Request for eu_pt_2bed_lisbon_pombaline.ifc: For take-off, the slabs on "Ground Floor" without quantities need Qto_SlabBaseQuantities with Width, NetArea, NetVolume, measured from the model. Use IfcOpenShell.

First a look at what the model holds.

```python
import ifcopenshell
import ifcopenshell.util.element
import ifcopenshell.util.unit

model = ifcopenshell.open("eu_pt_2bed_lisbon_pombaline.ifc")
print(model.schema)
for unit_type in ("LENGTHUNIT", "AREAUNIT", "VOLUMEUNIT"):
    print(unit_type, ifcopenshell.util.unit.calculate_unit_scale(model, unit_type))
storey = next(s for s in model.by_type("IfcBuildingStorey") if s.Name == "Ground Floor")
slabs = [e for e in ifcopenshell.util.element.get_decomposition(storey) if e.is_a("IfcSlab")]
for e in sorted(slabs, key=lambda e: e.id()):
    print(e.id(), e.is_a(), e.Name, list(ifcopenshell.util.element.get_psets(e, qtos_only=True)), sep=" | ")
```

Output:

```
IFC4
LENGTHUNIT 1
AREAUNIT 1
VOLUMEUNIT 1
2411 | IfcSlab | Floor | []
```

```python
import ifcopenshell
import ifcopenshell.api.pset
import ifcopenshell.geom
import ifcopenshell.util.element
import ifcopenshell.util.shape
import ifcopenshell.util.unit

model = ifcopenshell.open("eu_pt_2bed_lisbon_pombaline.ifc")
unit_scale = ifcopenshell.util.unit.calculate_unit_scale(model)
area_scale = ifcopenshell.util.unit.calculate_unit_scale(model, "AREAUNIT")
volume_scale = ifcopenshell.util.unit.calculate_unit_scale(model, "VOLUMEUNIT")
settings = ifcopenshell.geom.settings()

storey = next(s for s in model.by_type("IfcBuildingStorey") if s.Name == "Ground Floor")
slabs = [e for e in ifcopenshell.util.element.get_decomposition(storey) if e.is_a("IfcSlab")]

for e in sorted(slabs, key=lambda e: e.id()):
    if ifcopenshell.util.element.get_psets(e, qtos_only=True, should_inherit=False):
        continue
    # Geometry comes back in metres, in the element's own axes.
    shape = ifcopenshell.geom.create_shape(settings, e)
    values = {
        "Width": ifcopenshell.util.shape.get_z(shape.geometry) / unit_scale,
        "NetArea": ifcopenshell.util.shape.get_footprint_area(shape.geometry) / area_scale,
        "NetVolume": ifcopenshell.util.shape.get_volume(shape.geometry) / volume_scale,
    }
    qto = ifcopenshell.api.pset.add_qto(model, product=e, name="Qto_SlabBaseQuantities")
    ifcopenshell.api.pset.edit_qto(model, qto=qto, properties=values)
    print(e.id(), {k: round(v, 3) for k, v in values.items()})

model.write("eu_pt_2bed_lisbon_pombaline-out.ifc")
```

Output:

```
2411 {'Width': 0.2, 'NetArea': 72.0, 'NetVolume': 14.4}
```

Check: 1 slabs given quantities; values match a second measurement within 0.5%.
